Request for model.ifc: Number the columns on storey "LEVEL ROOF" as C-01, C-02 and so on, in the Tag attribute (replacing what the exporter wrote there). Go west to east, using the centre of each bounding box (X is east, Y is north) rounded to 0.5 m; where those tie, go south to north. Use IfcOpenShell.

First a look at what the model holds.

```python
import ifcopenshell
import ifcopenshell.util.element
import ifcopenshell.util.placement

model = ifcopenshell.open("model.ifc")
print(model.schema)
storey = next(s for s in model.by_type("IfcBuildingStorey") if s.Name == "LEVEL ROOF")
columns = [e for e in ifcopenshell.util.element.get_decomposition(storey) if e.is_a("IfcColumn")]
for e in sorted(columns, key=lambda e: e.id()):
    origin = ifcopenshell.util.placement.get_local_placement(e.ObjectPlacement)[:3, 3]
    print(e.id(), e.Tag, e.Name, origin.round(2) + 0.0, sep=" | ")
```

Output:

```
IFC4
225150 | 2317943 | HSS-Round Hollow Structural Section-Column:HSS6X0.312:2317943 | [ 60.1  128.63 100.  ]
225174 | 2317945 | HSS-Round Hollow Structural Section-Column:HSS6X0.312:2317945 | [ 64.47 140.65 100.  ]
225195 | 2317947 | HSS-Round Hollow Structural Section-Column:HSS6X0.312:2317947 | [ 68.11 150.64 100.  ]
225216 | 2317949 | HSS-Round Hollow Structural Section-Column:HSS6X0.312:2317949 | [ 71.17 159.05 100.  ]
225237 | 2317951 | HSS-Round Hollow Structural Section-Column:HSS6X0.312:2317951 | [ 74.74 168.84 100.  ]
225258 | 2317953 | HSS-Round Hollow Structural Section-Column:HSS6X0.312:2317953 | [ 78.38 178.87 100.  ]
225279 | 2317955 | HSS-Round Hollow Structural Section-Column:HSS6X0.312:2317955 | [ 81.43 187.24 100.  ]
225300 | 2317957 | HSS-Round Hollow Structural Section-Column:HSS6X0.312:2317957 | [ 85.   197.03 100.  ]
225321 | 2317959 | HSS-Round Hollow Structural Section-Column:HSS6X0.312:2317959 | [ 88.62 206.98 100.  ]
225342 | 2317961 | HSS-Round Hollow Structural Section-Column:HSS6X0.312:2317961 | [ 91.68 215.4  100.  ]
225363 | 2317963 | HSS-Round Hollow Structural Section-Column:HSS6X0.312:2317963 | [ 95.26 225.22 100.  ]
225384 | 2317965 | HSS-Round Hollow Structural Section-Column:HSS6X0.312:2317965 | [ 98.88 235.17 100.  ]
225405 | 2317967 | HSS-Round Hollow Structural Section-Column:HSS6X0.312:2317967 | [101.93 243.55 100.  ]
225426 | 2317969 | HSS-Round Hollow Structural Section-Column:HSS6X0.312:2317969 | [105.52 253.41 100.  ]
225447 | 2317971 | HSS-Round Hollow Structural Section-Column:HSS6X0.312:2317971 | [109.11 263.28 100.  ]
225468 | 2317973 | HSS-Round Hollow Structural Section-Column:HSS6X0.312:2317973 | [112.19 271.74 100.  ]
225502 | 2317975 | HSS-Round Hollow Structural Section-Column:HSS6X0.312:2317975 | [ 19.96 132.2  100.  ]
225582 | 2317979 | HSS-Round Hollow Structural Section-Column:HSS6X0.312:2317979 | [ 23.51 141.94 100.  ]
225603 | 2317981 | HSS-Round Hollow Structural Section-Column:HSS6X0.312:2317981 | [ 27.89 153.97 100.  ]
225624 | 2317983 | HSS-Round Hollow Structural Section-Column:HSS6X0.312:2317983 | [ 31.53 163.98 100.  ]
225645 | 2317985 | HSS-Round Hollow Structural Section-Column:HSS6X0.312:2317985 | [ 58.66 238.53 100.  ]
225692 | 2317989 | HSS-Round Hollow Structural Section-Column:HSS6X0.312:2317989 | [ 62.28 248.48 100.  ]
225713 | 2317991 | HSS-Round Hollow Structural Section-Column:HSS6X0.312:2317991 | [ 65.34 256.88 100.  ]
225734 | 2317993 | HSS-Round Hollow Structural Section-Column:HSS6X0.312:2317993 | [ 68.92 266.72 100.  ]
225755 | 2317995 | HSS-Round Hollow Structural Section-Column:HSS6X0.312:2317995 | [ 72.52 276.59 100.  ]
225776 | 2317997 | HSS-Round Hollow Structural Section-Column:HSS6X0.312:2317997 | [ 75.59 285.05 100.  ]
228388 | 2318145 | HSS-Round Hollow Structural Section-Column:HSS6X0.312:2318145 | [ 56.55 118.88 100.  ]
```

```python
import ifcopenshell
import ifcopenshell.geom
import ifcopenshell.util.element
import ifcopenshell.util.shape

model = ifcopenshell.open("model.ifc")
settings = ifcopenshell.geom.settings()
settings.set("use-world-coords", True)


def centre(element):
    shape = ifcopenshell.geom.create_shape(settings, element)
    return ifcopenshell.util.shape.get_bbox_centroid(shape.geometry)


storey = next(s for s in model.by_type("IfcBuildingStorey") if s.Name == "LEVEL ROOF")
columns = [e for e in ifcopenshell.util.element.get_decomposition(storey) if e.is_a("IfcColumn")]

# Insertion points can sit at a corner or the storey origin, so sort by the geometry (in metres).
centres = {e: centre(e) for e in columns}
columns.sort(key=lambda e: (round(centres[e][0] / 0.5), centres[e][1]))

for i, e in enumerate(columns, start=1):
    number = f"C-{i:02d}"
    e.Tag = number
    print(e.id(), number)

model.write("model_v2.ifc")
```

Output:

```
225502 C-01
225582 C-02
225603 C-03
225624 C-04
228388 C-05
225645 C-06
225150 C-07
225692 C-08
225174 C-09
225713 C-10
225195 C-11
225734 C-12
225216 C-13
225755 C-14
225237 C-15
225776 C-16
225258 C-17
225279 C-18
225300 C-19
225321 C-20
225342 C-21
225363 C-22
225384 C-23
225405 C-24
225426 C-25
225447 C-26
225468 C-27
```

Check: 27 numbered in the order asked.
